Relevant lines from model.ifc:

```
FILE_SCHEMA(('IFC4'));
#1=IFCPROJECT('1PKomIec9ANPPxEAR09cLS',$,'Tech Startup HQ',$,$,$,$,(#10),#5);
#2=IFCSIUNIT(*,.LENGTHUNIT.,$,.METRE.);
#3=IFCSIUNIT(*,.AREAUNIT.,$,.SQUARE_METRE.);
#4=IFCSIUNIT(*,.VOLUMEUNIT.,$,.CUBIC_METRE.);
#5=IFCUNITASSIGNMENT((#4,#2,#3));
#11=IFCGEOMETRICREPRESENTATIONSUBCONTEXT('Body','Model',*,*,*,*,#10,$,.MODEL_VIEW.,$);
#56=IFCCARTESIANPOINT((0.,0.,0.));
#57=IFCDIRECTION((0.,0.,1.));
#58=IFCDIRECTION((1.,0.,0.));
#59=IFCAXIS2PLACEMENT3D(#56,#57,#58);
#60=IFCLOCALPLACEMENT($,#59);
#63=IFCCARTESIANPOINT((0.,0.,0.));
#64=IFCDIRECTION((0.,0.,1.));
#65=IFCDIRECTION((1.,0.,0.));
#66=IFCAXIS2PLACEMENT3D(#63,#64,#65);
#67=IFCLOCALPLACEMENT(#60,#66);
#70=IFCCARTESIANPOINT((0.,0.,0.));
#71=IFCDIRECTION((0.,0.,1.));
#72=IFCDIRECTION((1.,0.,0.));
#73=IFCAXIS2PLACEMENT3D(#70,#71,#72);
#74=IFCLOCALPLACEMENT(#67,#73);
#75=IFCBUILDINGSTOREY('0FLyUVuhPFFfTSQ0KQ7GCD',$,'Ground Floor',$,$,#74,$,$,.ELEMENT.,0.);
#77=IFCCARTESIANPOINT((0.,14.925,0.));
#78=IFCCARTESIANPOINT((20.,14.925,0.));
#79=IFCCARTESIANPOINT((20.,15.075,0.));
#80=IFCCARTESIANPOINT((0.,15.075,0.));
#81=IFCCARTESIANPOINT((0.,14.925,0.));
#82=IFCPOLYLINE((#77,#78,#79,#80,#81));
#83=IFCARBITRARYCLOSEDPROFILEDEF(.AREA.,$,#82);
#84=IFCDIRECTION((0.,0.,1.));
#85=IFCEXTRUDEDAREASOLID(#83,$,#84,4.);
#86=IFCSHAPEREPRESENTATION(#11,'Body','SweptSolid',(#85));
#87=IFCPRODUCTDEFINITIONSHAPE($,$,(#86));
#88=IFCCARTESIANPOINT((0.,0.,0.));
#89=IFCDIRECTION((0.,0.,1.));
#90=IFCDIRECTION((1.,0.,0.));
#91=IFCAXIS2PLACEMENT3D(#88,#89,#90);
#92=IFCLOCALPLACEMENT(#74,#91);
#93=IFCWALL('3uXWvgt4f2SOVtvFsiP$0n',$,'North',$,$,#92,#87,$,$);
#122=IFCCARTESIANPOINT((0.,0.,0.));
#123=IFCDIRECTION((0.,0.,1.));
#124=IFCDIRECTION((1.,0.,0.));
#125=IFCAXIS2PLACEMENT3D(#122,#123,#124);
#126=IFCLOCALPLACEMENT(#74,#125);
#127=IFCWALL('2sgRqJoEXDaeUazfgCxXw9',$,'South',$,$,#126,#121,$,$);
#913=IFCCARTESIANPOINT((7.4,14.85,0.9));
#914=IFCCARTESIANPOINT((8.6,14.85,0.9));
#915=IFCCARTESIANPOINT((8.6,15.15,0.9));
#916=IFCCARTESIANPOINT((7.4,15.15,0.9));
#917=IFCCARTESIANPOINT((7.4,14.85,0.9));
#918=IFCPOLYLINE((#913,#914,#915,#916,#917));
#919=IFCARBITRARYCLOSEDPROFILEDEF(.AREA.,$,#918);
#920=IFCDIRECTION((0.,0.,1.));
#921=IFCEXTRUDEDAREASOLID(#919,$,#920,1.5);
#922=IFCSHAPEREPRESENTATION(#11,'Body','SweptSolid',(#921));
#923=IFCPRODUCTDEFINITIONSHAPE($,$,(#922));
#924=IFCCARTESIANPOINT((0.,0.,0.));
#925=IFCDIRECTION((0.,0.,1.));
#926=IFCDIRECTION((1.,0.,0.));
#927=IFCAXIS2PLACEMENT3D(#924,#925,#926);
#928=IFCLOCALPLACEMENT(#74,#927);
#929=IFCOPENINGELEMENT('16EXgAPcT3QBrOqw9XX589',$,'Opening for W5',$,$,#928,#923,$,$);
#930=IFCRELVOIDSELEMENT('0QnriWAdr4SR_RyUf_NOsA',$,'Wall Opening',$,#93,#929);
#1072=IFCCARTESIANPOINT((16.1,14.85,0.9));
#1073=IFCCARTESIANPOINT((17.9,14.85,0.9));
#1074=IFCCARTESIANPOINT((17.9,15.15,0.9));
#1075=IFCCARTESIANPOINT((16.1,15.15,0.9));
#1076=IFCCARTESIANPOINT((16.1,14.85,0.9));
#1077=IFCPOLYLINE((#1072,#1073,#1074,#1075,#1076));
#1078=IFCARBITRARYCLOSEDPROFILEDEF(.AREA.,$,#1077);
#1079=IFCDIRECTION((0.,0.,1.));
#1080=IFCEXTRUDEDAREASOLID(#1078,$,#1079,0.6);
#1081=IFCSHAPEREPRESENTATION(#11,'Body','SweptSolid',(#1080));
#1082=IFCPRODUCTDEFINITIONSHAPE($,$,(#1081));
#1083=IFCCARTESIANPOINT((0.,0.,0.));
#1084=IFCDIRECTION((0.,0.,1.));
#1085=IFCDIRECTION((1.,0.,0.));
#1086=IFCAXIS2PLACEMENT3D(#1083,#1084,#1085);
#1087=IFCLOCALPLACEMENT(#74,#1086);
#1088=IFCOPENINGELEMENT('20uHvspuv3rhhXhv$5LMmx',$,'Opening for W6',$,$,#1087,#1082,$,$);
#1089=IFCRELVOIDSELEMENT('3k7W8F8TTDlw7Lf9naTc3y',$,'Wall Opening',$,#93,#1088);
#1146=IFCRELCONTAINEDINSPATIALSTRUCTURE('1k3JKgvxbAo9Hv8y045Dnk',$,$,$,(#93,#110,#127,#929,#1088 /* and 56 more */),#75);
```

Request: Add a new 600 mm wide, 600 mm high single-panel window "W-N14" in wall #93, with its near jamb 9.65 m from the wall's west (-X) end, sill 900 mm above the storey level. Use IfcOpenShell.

```python
import numpy as np
import ifcopenshell
import ifcopenshell.api.feature
import ifcopenshell.api.geometry
import ifcopenshell.api.root
import ifcopenshell.api.spatial
import ifcopenshell.geom
import ifcopenshell.util.element
import ifcopenshell.util.placement
import ifcopenshell.util.representation
import ifcopenshell.util.shape
import ifcopenshell.util.unit

model = ifcopenshell.open("model.ifc")
unit_scale = ifcopenshell.util.unit.calculate_unit_scale(model)
settings = ifcopenshell.geom.settings()


def volume(element):
    """Net volume in cubic metres, openings subtracted."""
    shape = ifcopenshell.geom.create_shape(settings, element)
    return ifcopenshell.util.shape.get_volume(shape.geometry)


wall = model.by_guid("3uXWvgt4f2SOVtvFsiP$0n")
storey = ifcopenshell.util.element.get_container(wall, ifc_class="IfcBuildingStorey")
context = ifcopenshell.util.representation.get_context(model, "Model", "Body", "MODEL_VIEW")
before = volume(wall)

width, height, from_end, sill = 0.6, 0.6, 9.65, 0.9  # metres

# The wall runs along its own X axis, and the end named is its -X end.
wall_shape = ifcopenshell.geom.create_shape(settings, wall)
x, y, z = ifcopenshell.util.shape.get_vertices(wall_shape.geometry).T
start = x.min() + from_end
face, thickness = float(y.min()), float(y.max() - y.min())
wall_matrix = ifcopenshell.util.placement.get_local_placement(wall.ObjectPlacement)
level = ifcopenshell.util.placement.get_local_placement(storey.ObjectPlacement)[2, 3]


def in_wall(x, y):
    """Placement at x, y metres in the wall's axes, at sill height."""
    matrix = wall_matrix.copy()
    matrix[:, 3] = wall_matrix @ np.array([x / unit_scale, y / unit_scale, 0.0, 1.0])
    matrix[2, 3] = level + sill / unit_scale
    return matrix


# Opening: a box that overshoots both wall faces by 50 mm.
opening = ifcopenshell.api.root.create_entity(model, ifc_class="IfcOpeningElement", predefined_type="OPENING")
box = ifcopenshell.api.geometry.add_wall_representation(
    model, context=context, length=width, height=height, thickness=thickness + 0.1
)
ifcopenshell.api.geometry.assign_representation(model, product=opening, representation=box)
ifcopenshell.api.geometry.edit_object_placement(model, product=opening, matrix=in_wall(start, face - 0.05), is_si=False)
ifcopenshell.api.feature.add_feature(model, feature=opening, element=wall)

window = ifcopenshell.api.root.create_entity(model, ifc_class="IfcWindow", name="W-N14", predefined_type="WINDOW")
window.OverallWidth, window.OverallHeight = width / unit_scale, height / unit_scale
window.PartitioningType = "SINGLE_PANEL"
body = ifcopenshell.api.geometry.add_window_representation(
    model,
    context=context,
    overall_width=window.OverallWidth,
    overall_height=window.OverallHeight,
    partition_type="SINGLE_PANEL",
)
ifcopenshell.api.geometry.assign_representation(model, product=window, representation=body)
ifcopenshell.api.spatial.assign_container(model, products=[window], relating_structure=storey)
ifcopenshell.api.feature.add_filling(model, opening=opening, element=window)

# Centre the window in the wall's thickness.
ifcopenshell.api.geometry.edit_object_placement(model, product=window, matrix=in_wall(start, face), is_si=False)
window_shape = ifcopenshell.geom.create_shape(settings, window)
depth = ifcopenshell.util.shape.get_vertices(window_shape.geometry)[:, 1]
offset = face + thickness / 2 - (depth.min() + depth.max()) / 2
ifcopenshell.api.geometry.edit_object_placement(model, product=window, matrix=in_wall(start, offset), is_si=False)

after = volume(wall)

print(f"wall volume {before:.3f} -> {after:.3f} m3")

model.write("model_v2.ifc")
```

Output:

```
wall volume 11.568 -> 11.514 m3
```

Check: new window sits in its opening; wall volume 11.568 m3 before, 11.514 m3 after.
